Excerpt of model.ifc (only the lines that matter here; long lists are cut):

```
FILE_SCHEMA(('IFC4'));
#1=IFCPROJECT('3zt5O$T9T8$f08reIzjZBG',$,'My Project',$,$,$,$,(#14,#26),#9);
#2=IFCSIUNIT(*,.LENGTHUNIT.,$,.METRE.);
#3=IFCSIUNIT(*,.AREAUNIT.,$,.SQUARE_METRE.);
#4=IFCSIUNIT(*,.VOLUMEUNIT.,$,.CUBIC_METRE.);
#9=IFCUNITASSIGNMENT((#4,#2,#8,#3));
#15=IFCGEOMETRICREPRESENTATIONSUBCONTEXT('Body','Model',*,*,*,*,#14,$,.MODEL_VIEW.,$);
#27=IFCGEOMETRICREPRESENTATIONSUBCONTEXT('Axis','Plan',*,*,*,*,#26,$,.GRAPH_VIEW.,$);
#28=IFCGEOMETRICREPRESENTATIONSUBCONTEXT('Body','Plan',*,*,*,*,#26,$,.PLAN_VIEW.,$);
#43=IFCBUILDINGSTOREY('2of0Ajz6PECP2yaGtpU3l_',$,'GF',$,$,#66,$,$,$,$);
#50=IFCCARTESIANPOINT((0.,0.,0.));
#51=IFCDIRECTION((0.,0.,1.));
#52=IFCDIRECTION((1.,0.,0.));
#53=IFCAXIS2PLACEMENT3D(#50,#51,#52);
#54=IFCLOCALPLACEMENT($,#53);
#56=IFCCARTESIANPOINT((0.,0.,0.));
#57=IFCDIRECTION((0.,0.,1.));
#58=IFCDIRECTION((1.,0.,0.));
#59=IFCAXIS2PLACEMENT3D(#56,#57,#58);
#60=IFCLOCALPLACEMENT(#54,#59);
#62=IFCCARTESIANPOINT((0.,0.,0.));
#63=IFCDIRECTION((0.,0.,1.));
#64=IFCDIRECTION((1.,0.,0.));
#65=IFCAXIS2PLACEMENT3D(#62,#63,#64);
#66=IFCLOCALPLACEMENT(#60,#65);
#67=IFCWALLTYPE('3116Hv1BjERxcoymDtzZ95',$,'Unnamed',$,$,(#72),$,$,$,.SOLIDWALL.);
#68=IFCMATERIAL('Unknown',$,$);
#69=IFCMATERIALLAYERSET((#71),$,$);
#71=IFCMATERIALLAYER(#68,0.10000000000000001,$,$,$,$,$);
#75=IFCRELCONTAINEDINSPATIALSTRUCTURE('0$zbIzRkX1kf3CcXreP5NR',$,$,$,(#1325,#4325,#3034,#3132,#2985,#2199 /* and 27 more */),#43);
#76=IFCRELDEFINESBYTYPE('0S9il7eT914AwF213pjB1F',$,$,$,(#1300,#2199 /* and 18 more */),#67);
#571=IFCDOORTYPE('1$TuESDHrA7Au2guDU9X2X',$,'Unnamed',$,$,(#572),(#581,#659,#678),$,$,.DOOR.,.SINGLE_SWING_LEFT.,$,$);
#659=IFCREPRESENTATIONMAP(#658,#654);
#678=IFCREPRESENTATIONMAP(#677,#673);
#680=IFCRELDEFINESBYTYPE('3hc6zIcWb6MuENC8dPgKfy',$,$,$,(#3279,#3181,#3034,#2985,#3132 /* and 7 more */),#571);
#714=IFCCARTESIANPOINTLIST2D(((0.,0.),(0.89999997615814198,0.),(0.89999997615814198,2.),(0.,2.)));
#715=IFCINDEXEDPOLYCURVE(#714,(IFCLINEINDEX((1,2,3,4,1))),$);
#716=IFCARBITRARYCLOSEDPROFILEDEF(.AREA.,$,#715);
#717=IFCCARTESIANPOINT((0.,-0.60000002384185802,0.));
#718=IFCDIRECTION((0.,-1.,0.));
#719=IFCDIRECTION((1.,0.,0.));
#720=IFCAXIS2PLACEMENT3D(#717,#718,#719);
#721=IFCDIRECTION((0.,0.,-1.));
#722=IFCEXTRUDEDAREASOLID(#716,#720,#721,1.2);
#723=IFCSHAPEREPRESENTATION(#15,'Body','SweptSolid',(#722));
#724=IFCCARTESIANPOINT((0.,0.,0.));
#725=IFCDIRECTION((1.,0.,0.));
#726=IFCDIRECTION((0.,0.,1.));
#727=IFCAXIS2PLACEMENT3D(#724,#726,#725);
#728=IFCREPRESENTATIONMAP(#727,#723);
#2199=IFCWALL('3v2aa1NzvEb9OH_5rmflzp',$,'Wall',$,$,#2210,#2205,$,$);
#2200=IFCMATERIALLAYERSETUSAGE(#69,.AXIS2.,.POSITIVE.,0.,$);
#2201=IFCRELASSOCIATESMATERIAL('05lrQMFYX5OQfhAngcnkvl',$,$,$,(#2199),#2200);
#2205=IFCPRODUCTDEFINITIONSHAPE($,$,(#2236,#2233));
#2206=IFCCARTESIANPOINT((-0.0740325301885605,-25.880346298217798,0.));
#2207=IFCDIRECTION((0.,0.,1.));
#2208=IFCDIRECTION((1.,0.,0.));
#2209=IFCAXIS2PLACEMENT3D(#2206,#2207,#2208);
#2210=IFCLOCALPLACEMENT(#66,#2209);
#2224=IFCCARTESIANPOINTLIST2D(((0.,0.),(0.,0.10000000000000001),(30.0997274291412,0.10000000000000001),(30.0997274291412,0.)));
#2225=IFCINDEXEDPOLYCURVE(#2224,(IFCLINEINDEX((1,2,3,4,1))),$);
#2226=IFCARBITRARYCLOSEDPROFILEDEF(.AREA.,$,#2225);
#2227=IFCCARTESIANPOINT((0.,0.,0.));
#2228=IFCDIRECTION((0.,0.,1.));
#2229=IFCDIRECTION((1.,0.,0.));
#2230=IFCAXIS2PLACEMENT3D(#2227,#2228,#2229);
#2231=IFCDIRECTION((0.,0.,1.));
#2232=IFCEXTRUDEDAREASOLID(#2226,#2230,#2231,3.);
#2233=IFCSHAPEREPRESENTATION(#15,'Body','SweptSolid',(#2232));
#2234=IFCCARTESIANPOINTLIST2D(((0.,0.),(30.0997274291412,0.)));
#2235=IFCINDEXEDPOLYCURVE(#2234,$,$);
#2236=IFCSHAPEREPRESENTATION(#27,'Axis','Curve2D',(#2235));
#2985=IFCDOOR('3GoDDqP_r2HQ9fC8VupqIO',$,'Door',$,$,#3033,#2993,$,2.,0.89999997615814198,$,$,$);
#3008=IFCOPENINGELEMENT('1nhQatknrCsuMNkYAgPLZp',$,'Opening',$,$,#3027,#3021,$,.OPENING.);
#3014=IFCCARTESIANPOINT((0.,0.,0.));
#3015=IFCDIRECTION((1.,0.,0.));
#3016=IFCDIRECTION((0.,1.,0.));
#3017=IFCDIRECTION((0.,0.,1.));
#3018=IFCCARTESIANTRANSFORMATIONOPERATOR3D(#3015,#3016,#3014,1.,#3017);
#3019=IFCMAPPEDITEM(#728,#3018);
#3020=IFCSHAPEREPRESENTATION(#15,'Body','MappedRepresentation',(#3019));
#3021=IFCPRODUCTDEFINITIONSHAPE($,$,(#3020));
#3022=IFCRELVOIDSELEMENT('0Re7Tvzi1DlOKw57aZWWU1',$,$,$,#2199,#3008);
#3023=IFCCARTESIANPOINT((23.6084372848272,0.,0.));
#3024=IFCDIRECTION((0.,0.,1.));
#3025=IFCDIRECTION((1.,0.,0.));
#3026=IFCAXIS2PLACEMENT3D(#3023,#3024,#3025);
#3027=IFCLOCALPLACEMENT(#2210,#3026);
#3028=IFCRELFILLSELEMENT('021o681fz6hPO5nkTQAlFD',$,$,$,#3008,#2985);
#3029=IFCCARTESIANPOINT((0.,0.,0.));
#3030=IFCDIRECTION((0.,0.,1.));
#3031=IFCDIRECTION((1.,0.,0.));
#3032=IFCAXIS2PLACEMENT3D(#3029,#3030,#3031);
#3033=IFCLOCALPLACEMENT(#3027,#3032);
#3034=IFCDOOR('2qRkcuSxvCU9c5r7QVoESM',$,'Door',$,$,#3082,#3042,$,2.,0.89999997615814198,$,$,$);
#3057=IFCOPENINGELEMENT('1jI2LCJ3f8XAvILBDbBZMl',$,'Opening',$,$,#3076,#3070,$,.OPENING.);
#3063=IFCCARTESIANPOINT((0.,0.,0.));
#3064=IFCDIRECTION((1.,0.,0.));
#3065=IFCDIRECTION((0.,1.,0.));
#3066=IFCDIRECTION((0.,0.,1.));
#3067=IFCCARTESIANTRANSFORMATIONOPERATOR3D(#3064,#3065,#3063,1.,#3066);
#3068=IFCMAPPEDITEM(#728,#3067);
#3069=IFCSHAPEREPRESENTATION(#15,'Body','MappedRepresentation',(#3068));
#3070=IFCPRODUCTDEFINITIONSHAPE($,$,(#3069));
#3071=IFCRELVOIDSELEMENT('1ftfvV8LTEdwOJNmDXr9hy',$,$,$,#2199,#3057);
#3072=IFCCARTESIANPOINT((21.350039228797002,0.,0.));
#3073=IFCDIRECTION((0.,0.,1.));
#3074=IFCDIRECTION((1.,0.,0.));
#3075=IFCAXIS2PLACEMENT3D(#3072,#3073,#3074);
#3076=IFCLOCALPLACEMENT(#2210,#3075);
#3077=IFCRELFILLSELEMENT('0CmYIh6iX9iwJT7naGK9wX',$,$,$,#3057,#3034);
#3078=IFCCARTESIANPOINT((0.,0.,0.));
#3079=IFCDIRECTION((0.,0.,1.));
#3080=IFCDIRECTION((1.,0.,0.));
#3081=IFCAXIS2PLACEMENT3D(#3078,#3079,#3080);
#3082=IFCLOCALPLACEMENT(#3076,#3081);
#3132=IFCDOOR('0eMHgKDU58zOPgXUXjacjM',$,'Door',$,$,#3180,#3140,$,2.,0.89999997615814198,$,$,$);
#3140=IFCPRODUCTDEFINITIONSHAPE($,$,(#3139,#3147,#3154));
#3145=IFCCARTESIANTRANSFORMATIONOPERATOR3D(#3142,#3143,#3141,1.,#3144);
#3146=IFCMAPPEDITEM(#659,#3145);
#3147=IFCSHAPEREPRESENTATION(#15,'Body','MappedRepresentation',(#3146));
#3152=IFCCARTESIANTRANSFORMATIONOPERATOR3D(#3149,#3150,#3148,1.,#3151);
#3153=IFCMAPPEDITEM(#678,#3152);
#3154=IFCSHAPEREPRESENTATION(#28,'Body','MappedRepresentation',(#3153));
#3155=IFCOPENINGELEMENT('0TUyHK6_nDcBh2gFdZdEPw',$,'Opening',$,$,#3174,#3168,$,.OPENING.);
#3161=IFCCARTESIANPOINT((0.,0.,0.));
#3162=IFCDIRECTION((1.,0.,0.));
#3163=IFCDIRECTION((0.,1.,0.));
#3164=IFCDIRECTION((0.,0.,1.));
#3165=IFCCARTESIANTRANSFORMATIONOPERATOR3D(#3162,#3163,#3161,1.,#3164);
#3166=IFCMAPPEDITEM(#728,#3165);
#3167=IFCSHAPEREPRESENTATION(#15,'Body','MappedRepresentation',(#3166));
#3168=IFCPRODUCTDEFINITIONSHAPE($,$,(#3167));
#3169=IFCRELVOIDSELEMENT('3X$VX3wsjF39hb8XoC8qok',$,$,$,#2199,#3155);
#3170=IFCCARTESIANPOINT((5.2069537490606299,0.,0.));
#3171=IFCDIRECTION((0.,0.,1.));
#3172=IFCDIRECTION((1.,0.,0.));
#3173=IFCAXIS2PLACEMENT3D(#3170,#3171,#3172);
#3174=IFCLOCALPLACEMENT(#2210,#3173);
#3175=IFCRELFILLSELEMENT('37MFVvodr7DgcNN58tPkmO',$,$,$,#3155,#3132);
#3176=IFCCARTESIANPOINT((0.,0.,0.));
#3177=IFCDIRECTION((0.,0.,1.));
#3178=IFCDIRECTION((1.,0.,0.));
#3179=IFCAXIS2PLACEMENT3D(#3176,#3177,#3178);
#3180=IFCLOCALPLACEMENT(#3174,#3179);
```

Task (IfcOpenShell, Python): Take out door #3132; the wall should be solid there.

```python
import ifcopenshell
import ifcopenshell.api.feature
import ifcopenshell.api.root
import ifcopenshell.geom
import ifcopenshell.util.shape

model = ifcopenshell.open("model.ifc")
settings = ifcopenshell.geom.settings()


def volume(element):
    """Net volume in cubic metres, openings subtracted."""
    shape = ifcopenshell.geom.create_shape(settings, element)
    return ifcopenshell.util.shape.get_volume(shape.geometry)


door = model.by_guid("0eMHgKDU58zOPgXUXjacjM")
opening = door.FillsVoids[0].RelatingOpeningElement
wall = opening.VoidsElements[0].RelatingBuildingElement
before = volume(wall)

ifcopenshell.api.root.remove_product(model, product=door)
ifcopenshell.api.feature.remove_feature(model, feature=opening)

after = volume(wall)

print(f"wall volume {before:.3f} -> {after:.3f} m3")

model.write("model_v2.ifc")
```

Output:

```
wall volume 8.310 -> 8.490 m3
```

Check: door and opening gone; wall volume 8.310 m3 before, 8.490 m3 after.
